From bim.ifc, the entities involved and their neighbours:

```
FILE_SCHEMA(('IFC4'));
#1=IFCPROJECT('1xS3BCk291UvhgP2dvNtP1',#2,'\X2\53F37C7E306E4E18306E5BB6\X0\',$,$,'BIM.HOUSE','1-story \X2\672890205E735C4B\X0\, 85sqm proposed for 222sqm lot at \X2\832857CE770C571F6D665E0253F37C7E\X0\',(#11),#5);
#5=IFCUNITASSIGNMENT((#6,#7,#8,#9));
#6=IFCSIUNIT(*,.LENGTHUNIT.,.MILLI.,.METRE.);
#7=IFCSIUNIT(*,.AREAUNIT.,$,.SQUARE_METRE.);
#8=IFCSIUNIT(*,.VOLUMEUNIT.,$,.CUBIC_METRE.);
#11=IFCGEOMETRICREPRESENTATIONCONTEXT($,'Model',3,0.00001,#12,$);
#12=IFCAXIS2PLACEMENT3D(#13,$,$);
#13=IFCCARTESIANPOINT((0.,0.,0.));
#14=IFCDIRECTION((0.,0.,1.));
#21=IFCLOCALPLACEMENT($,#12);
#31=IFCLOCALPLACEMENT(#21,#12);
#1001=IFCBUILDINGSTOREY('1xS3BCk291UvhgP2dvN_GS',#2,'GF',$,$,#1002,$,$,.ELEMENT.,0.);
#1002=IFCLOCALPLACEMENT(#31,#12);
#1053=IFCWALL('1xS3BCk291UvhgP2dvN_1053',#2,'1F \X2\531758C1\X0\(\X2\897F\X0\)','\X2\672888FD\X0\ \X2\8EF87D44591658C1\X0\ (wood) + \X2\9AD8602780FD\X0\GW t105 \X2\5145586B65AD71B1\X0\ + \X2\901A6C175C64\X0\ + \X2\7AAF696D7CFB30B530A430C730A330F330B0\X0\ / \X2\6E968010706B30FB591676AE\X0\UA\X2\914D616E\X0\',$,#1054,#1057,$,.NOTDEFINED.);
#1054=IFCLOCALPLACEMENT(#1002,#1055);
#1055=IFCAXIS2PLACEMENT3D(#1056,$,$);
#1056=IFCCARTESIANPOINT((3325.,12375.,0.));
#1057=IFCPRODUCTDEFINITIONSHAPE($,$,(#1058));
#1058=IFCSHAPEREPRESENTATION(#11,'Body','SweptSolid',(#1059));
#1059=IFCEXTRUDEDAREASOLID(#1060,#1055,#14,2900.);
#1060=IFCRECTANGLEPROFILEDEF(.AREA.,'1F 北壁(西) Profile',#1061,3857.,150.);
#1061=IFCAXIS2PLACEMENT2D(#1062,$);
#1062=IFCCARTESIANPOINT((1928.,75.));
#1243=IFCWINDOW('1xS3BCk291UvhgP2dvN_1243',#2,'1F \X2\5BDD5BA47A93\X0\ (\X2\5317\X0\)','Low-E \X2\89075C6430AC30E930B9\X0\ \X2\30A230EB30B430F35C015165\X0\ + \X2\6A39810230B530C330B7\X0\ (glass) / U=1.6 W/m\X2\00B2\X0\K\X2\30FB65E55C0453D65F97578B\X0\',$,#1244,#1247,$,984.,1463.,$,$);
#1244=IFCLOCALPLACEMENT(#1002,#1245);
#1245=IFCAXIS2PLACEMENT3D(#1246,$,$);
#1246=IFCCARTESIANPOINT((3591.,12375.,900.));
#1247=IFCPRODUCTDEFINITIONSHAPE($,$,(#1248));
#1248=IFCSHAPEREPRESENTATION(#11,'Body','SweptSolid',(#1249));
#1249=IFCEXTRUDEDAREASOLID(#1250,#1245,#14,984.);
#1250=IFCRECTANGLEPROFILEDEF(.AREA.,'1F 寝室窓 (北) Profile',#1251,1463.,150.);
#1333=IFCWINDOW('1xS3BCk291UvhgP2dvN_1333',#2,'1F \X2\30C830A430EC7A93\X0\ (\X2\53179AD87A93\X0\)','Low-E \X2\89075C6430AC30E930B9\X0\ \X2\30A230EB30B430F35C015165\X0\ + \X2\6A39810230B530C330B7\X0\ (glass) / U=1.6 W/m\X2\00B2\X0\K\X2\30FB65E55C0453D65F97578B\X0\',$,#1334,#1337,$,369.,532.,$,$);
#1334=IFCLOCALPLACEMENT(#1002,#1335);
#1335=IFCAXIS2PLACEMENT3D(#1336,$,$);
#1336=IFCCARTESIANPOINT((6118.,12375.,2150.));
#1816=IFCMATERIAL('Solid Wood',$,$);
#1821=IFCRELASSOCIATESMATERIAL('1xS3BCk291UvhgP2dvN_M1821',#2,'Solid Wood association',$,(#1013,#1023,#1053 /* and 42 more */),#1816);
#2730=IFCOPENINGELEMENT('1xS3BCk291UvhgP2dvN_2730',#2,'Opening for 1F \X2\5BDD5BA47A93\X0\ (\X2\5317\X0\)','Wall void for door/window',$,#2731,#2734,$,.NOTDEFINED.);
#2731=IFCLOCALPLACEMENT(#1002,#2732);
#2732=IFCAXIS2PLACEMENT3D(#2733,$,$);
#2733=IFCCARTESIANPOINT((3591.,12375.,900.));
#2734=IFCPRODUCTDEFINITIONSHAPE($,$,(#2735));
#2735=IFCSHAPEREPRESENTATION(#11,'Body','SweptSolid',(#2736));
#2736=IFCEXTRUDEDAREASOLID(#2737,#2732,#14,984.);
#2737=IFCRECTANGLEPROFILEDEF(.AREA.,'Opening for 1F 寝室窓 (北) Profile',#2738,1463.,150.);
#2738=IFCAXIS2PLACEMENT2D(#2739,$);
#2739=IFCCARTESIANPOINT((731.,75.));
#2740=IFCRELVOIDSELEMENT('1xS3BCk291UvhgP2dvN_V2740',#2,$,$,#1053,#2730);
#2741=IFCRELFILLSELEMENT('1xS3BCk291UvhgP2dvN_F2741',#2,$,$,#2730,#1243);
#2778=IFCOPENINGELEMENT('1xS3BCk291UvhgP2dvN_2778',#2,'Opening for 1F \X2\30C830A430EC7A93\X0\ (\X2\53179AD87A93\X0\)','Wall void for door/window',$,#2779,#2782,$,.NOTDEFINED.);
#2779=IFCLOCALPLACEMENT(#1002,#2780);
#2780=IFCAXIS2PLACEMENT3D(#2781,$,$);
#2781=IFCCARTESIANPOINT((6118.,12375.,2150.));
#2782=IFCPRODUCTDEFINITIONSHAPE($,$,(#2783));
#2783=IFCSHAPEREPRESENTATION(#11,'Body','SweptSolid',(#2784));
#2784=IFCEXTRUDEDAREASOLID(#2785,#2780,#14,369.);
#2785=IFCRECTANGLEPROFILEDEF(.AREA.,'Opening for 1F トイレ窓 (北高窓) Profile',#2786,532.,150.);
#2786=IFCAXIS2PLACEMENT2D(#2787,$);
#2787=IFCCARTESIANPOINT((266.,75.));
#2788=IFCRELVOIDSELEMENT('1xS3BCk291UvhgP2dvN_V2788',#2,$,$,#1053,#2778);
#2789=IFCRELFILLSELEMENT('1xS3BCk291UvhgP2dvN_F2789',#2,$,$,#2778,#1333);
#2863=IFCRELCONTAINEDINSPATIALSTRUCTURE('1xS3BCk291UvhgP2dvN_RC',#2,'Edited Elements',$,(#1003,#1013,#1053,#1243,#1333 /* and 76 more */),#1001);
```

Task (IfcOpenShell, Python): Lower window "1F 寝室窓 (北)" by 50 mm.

```python
import numpy as np
import ifcopenshell
import ifcopenshell.api.geometry
import ifcopenshell.util.placement
import ifcopenshell.util.unit

model = ifcopenshell.open("bim.ifc")
unit_scale = ifcopenshell.util.unit.calculate_unit_scale(model)

window = model.by_guid("1xS3BCk291UvhgP2dvN_1243")
opening = window.FillsVoids[0].RelatingOpeningElement
dz = -50.0

shift = np.array([0.0, 0.0, dz])
# The window is not placed relative to its opening, so move both.
for product in (opening, window):
    matrix = ifcopenshell.util.placement.get_local_placement(product.ObjectPlacement)
    matrix[:3, 3] += shift
    ifcopenshell.api.geometry.edit_object_placement(model, product=product, matrix=matrix, is_si=False)

print(f"moved by {dz * unit_scale:+.3f} m")

model.write("bim_v2.ifc")
```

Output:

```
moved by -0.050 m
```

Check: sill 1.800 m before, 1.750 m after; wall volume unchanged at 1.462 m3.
